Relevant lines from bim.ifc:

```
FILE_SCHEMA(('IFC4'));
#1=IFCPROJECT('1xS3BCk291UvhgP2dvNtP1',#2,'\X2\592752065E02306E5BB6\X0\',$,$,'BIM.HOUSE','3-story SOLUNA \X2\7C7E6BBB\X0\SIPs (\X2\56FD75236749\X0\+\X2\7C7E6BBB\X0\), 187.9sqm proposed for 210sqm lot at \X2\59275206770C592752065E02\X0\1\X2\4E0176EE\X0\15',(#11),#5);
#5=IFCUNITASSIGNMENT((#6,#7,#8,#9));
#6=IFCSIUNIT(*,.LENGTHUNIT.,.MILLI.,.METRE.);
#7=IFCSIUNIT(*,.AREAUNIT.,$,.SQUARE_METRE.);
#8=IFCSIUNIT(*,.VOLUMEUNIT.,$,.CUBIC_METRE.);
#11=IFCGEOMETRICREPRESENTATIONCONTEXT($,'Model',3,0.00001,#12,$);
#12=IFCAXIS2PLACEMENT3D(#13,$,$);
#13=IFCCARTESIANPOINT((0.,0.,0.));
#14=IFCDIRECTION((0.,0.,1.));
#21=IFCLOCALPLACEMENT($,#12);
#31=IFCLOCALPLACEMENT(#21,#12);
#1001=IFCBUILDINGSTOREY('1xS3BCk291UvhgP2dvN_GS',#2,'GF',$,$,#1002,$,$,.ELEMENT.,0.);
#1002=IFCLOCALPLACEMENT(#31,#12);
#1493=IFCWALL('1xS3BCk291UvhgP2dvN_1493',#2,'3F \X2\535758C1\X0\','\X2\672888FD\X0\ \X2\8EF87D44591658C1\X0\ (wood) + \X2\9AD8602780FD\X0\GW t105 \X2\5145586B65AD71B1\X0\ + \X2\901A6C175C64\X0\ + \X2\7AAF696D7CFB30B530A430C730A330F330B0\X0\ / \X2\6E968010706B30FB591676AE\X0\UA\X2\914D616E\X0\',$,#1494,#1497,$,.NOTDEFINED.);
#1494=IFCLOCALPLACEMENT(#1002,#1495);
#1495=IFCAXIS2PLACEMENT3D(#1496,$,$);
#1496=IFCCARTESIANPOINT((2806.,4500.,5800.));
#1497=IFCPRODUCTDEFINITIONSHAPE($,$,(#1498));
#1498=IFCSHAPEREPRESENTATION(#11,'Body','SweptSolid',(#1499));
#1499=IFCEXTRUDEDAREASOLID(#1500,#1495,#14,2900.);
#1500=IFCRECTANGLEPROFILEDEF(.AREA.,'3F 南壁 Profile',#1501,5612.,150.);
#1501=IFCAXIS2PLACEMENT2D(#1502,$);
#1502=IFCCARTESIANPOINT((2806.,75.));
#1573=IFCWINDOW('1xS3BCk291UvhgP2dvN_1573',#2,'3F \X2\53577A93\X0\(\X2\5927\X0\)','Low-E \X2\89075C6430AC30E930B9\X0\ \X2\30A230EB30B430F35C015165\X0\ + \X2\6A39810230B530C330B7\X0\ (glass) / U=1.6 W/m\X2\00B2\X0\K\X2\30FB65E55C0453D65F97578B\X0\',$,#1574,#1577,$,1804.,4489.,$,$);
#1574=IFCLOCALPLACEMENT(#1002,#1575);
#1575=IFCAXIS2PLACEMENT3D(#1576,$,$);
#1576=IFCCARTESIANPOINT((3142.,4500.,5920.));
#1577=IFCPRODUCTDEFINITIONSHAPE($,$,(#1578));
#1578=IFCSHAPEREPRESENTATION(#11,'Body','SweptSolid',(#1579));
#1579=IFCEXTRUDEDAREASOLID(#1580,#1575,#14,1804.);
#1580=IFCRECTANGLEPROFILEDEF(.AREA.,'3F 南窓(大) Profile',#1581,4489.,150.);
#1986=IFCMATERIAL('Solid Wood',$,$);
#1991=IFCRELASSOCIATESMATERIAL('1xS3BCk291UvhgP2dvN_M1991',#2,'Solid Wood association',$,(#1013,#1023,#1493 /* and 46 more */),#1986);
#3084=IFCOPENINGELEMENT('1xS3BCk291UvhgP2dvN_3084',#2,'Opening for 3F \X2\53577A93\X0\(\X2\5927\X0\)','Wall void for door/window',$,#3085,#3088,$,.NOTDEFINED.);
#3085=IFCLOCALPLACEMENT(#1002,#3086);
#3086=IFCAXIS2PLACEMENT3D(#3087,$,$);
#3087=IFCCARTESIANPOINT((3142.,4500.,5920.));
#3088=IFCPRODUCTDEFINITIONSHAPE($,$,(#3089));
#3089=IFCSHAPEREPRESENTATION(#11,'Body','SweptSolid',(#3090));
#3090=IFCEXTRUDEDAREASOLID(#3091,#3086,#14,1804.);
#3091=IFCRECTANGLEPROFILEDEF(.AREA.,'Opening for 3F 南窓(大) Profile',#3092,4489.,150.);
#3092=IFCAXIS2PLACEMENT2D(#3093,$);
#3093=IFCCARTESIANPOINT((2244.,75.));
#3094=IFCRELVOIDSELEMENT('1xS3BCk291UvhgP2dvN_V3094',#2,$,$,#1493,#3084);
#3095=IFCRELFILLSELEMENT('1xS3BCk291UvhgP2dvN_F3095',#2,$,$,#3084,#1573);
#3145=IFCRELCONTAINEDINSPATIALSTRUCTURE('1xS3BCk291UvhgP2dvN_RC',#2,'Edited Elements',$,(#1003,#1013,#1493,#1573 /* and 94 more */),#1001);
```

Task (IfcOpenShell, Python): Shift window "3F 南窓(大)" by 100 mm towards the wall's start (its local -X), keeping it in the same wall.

```python
import ifcopenshell
import ifcopenshell.api.geometry
import ifcopenshell.util.placement

model = ifcopenshell.open("bim.ifc")

window = model.by_guid("1xS3BCk291UvhgP2dvN_1573")
opening = window.FillsVoids[0].RelatingOpeningElement
wall = opening.VoidsElements[0].RelatingBuildingElement

wall_matrix = ifcopenshell.util.placement.get_local_placement(wall.ObjectPlacement)
shift = wall_matrix[:3, 0] * -100.0
before = ifcopenshell.util.placement.get_local_placement(window.ObjectPlacement)[:3, 3].copy()

# The window is not placed relative to its opening, so move both.
for product in (opening, window):
    matrix = ifcopenshell.util.placement.get_local_placement(product.ObjectPlacement)
    matrix[:3, 3] += shift
    ifcopenshell.api.geometry.edit_object_placement(model, product=product, matrix=matrix, is_si=False)

after = ifcopenshell.util.placement.get_local_placement(window.ObjectPlacement)[:3, 3]
print("window moved by", (after - before).round(3) + 0.0)

model.write("bim_v2.ifc")
```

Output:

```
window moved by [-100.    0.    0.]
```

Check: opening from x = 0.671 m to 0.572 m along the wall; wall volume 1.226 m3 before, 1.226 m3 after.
